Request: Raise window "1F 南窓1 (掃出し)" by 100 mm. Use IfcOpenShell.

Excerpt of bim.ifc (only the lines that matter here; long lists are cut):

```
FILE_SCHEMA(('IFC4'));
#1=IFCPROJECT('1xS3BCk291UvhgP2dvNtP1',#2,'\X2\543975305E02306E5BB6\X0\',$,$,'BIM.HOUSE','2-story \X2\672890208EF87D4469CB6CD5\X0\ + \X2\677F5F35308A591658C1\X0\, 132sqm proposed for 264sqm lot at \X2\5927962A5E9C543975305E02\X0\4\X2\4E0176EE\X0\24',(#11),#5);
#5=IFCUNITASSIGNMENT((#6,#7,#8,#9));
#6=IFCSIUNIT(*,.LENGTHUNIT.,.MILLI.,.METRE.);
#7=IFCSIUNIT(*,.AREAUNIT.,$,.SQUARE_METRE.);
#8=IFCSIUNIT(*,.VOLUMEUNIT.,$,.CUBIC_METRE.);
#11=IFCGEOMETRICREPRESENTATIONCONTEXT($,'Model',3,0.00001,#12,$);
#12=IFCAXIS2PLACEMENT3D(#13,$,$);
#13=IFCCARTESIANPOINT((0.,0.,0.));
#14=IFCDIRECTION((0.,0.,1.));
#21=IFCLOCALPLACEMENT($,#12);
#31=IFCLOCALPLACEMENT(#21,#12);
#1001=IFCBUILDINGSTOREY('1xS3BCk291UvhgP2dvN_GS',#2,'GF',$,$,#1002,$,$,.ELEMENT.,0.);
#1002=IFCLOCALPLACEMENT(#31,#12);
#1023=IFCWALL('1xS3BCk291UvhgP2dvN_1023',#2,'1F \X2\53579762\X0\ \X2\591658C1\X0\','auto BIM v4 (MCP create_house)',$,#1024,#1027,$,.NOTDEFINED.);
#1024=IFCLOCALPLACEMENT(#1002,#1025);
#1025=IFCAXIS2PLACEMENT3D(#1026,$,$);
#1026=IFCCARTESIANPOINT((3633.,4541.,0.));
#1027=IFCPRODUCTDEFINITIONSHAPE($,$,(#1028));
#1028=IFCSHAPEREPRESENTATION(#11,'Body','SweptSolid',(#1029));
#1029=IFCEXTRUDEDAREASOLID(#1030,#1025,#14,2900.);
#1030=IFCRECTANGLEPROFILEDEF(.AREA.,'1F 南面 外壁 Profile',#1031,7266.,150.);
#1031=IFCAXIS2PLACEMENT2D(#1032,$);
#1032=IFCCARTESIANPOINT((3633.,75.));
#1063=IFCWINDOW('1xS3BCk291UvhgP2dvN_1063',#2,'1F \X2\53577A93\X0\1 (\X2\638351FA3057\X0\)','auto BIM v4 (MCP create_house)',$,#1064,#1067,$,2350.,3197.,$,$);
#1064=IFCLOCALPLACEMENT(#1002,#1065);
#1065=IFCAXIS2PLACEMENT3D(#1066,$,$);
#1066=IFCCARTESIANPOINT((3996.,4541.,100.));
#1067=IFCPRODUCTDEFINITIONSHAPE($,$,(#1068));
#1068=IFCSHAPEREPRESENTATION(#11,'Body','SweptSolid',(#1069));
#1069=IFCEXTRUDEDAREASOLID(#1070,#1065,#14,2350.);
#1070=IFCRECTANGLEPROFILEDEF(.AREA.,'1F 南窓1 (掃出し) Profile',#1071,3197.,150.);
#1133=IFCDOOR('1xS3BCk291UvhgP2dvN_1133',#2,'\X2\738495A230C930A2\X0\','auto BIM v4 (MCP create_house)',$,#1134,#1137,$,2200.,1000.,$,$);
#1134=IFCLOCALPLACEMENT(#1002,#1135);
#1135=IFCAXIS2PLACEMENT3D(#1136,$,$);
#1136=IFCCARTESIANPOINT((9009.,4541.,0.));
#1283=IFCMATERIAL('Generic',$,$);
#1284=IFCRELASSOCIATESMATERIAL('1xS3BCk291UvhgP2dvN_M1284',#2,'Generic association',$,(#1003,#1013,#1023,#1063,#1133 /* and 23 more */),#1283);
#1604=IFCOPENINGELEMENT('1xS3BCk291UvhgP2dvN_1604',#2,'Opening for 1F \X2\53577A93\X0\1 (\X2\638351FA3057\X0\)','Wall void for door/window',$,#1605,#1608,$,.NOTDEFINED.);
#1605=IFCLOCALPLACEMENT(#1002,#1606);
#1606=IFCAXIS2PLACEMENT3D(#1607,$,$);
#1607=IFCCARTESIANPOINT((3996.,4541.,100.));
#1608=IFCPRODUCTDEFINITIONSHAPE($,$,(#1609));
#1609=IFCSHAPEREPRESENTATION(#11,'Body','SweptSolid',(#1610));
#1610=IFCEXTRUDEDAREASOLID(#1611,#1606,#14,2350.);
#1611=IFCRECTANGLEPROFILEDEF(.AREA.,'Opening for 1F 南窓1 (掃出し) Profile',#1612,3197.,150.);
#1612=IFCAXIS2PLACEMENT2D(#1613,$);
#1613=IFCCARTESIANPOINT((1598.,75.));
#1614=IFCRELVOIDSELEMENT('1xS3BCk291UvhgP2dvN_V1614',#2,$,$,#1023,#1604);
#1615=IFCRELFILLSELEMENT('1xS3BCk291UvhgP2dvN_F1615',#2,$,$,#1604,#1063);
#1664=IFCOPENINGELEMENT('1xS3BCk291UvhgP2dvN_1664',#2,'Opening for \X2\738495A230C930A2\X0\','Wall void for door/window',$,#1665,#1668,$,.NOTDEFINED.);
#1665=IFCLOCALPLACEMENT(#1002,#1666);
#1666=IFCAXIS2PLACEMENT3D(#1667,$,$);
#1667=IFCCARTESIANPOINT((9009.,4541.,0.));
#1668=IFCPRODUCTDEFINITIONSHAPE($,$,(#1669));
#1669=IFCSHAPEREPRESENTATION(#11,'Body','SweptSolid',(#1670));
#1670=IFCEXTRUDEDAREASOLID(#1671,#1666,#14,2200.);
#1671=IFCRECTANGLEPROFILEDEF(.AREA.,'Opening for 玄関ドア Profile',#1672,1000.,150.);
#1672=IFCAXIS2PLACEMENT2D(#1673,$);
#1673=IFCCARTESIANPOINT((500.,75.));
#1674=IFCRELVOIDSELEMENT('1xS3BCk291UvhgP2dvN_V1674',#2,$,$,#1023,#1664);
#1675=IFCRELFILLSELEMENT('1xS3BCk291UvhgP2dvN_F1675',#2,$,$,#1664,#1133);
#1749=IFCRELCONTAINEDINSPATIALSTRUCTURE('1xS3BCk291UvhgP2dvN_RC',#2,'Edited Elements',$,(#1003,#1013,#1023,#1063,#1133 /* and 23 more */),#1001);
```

```python
import numpy as np
import ifcopenshell
import ifcopenshell.api.geometry
import ifcopenshell.util.placement
import ifcopenshell.util.unit

model = ifcopenshell.open("bim.ifc")
unit_scale = ifcopenshell.util.unit.calculate_unit_scale(model)

window = model.by_guid("1xS3BCk291UvhgP2dvN_1063")
opening = window.FillsVoids[0].RelatingOpeningElement
dz = 0.1 / unit_scale

shift = np.array([0.0, 0.0, dz])
# The window is not placed relative to its opening, so move both.
for product in (opening, window):
    matrix = ifcopenshell.util.placement.get_local_placement(product.ObjectPlacement)
    matrix[:3, 3] += shift
    ifcopenshell.api.geometry.edit_object_placement(model, product=product, matrix=matrix, is_si=False)

print(f"moved by {dz * unit_scale:+.3f} m")

model.write("bim-out.ifc")
```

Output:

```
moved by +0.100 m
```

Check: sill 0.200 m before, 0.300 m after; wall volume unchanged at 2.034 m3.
